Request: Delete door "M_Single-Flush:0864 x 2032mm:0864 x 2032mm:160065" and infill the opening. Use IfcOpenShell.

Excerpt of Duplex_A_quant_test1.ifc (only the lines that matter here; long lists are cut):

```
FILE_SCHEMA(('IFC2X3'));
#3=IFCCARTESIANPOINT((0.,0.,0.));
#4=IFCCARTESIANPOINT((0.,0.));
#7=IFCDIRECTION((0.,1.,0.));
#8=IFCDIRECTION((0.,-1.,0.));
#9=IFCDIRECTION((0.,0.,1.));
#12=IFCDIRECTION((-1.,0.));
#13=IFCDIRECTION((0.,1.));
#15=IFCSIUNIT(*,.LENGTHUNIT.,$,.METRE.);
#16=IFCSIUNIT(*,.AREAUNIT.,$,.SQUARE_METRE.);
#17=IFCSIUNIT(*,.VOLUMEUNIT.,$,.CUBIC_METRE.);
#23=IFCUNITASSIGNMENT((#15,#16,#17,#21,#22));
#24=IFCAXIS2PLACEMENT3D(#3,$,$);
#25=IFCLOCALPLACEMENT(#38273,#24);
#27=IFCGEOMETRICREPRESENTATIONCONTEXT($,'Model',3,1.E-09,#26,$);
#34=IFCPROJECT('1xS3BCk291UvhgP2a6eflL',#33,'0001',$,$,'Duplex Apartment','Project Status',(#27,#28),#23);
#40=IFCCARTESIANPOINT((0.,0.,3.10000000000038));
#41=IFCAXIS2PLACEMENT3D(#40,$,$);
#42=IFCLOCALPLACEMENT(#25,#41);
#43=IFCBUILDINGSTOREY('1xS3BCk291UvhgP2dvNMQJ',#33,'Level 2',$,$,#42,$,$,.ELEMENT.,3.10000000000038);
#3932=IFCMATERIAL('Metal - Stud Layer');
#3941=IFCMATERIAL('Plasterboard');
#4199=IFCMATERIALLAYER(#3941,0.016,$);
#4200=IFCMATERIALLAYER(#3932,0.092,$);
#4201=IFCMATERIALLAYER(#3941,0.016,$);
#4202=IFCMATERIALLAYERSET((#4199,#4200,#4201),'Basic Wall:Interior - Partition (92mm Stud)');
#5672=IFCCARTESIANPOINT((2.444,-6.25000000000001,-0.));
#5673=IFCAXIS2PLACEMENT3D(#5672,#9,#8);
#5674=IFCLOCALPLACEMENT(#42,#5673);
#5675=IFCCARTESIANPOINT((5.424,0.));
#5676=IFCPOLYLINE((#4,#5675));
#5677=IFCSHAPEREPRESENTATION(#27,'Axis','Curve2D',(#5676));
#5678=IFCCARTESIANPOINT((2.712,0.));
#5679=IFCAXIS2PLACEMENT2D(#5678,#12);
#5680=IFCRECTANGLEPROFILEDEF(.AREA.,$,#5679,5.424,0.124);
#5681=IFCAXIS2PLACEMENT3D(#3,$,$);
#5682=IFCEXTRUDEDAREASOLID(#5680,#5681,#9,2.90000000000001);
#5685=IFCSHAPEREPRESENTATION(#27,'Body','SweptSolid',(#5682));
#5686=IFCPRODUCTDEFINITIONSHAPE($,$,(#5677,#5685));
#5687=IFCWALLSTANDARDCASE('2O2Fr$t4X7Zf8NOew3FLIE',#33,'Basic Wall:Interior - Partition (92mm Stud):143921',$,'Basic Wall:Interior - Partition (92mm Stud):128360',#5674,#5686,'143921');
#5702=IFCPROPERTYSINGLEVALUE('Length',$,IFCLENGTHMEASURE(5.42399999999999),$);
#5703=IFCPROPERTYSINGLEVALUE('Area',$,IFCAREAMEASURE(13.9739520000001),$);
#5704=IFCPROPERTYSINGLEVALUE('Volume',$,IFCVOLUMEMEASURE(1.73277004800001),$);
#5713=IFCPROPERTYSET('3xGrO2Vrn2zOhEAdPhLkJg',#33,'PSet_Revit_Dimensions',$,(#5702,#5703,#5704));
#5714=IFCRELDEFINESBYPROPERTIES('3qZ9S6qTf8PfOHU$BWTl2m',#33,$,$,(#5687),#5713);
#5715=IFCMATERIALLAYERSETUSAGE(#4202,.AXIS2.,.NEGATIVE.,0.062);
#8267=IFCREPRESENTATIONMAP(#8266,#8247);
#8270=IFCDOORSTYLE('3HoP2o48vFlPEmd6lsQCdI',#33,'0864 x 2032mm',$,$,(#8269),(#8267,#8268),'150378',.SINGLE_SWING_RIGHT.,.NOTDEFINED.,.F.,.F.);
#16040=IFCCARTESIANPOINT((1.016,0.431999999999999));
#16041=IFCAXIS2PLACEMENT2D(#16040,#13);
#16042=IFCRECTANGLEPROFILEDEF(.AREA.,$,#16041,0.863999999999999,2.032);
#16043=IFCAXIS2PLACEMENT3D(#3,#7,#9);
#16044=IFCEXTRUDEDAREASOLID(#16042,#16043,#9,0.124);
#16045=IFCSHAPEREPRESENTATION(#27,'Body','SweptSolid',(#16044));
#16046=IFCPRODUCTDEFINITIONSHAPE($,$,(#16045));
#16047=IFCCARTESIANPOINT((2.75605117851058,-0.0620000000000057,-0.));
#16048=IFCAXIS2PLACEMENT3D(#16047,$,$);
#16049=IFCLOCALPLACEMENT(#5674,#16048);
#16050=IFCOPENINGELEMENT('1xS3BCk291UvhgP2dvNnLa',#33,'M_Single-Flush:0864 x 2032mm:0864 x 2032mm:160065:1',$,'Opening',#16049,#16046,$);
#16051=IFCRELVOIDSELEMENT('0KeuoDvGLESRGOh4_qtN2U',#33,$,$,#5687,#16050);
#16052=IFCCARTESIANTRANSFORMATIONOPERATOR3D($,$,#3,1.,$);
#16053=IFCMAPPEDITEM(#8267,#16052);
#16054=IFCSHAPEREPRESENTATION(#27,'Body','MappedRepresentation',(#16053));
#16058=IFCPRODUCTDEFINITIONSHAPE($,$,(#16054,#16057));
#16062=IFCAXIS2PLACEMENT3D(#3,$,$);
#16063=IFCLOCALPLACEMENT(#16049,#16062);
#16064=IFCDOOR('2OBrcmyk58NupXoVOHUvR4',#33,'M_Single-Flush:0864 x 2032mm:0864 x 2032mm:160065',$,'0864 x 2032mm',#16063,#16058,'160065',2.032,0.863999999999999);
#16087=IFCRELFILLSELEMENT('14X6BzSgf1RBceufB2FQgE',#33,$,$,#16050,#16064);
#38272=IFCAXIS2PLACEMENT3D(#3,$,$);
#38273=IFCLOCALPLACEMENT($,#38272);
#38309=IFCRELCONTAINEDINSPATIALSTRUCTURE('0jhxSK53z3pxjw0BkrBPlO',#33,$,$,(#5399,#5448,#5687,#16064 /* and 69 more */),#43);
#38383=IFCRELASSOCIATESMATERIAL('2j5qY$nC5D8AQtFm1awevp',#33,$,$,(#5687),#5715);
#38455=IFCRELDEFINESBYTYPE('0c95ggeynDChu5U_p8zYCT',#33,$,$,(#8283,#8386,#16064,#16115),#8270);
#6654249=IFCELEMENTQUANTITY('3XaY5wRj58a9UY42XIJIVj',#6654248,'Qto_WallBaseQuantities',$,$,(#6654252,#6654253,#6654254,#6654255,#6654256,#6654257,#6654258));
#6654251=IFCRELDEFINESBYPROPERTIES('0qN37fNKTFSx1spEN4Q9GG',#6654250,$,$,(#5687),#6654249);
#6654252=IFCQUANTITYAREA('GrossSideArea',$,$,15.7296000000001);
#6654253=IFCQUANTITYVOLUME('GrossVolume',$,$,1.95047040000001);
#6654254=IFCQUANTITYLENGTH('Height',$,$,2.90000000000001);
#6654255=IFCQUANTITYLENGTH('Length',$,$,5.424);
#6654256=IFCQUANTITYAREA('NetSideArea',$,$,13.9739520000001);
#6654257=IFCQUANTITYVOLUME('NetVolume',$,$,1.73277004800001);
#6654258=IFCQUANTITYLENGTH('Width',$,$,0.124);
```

```python
import ifcopenshell
import ifcopenshell.api.feature
import ifcopenshell.api.pset
import ifcopenshell.api.root
import ifcopenshell.geom
import ifcopenshell.util.element
import ifcopenshell.util.shape
import ifcopenshell.util.unit

model = ifcopenshell.open("Duplex_A_quant_test1.ifc")
area_scale = ifcopenshell.util.unit.calculate_unit_scale(model, "AREAUNIT")
volume_scale = ifcopenshell.util.unit.calculate_unit_scale(model, "VOLUMEUNIT")
settings = ifcopenshell.geom.settings()


def volume(element):
    """Net volume in cubic metres, openings subtracted."""
    shape = ifcopenshell.geom.create_shape(settings, element)
    return ifcopenshell.util.shape.get_volume(shape.geometry)


door = model.by_id(16064)
opening = door.FillsVoids[0].RelatingOpeningElement
wall = opening.VoidsElements[0].RelatingBuildingElement
before = volume(wall)

ifcopenshell.api.root.remove_product(model, product=door)
ifcopenshell.api.feature.remove_feature(model, feature=opening)

after = volume(wall)
thickness = 0.124  # wall thickness in metres

# Update the wall's stored quantities.
pset = model.by_id(ifcopenshell.util.element.get_pset(wall, "PSet_Revit_Dimensions", should_inherit=False)["id"])
ifcopenshell.api.pset.edit_pset(model, pset=pset, properties={
    "Area": model.create_entity("IfcAreaMeasure", after / thickness / area_scale),
    "Volume": model.create_entity("IfcVolumeMeasure", after / volume_scale),
})
qto = model.by_id(ifcopenshell.util.element.get_pset(wall, "Qto_WallBaseQuantities", should_inherit=False)["id"])
ifcopenshell.api.pset.edit_qto(model, qto=qto, properties={
    "NetSideArea": after / thickness / area_scale,
    "NetVolume": after / volume_scale,
})

print(f"wall volume {before:.3f} -> {after:.3f} m3")

model.write("Duplex_A_quant_test1_rev.ifc")
```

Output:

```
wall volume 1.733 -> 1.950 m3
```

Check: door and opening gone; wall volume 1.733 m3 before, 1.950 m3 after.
